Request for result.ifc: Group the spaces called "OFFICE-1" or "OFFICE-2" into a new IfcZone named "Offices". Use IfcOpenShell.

First a look at what the model holds.

```python
import ifcopenshell

model = ifcopenshell.open("result.ifc")
print(model.schema)
seen = {}
for space in model.by_type("IfcSpace"):
    seen[space.Name] = seen.get(space.Name, 0) + 1
for name, count in sorted(seen.items(), key=str):
    print(count, "x", name)
print("zones:", [z.Name for z in model.by_type("IfcZone")][:20])
```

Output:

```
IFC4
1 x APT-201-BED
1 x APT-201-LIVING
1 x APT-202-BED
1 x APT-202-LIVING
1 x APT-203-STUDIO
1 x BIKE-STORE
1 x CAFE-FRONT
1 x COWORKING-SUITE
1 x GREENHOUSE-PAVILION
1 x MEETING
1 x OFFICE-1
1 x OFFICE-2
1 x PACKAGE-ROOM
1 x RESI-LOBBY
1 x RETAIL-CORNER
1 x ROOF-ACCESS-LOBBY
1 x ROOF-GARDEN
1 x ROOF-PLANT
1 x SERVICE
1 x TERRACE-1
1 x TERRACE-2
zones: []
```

```python
import ifcopenshell
import ifcopenshell.api.group
import ifcopenshell.api.root

model = ifcopenshell.open("result.ifc")

names = {"OFFICE-1", "OFFICE-2"}
spaces = [s for s in model.by_type("IfcSpace") if s.Name in names]

zone = ifcopenshell.api.root.create_entity(model, ifc_class="IfcZone", name="Offices")
ifcopenshell.api.group.assign_group(model, products=spaces, group=zone)
print(len(spaces), "spaces in", zone.Name)

model.write("result_v2.ifc")
```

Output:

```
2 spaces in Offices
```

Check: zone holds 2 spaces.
